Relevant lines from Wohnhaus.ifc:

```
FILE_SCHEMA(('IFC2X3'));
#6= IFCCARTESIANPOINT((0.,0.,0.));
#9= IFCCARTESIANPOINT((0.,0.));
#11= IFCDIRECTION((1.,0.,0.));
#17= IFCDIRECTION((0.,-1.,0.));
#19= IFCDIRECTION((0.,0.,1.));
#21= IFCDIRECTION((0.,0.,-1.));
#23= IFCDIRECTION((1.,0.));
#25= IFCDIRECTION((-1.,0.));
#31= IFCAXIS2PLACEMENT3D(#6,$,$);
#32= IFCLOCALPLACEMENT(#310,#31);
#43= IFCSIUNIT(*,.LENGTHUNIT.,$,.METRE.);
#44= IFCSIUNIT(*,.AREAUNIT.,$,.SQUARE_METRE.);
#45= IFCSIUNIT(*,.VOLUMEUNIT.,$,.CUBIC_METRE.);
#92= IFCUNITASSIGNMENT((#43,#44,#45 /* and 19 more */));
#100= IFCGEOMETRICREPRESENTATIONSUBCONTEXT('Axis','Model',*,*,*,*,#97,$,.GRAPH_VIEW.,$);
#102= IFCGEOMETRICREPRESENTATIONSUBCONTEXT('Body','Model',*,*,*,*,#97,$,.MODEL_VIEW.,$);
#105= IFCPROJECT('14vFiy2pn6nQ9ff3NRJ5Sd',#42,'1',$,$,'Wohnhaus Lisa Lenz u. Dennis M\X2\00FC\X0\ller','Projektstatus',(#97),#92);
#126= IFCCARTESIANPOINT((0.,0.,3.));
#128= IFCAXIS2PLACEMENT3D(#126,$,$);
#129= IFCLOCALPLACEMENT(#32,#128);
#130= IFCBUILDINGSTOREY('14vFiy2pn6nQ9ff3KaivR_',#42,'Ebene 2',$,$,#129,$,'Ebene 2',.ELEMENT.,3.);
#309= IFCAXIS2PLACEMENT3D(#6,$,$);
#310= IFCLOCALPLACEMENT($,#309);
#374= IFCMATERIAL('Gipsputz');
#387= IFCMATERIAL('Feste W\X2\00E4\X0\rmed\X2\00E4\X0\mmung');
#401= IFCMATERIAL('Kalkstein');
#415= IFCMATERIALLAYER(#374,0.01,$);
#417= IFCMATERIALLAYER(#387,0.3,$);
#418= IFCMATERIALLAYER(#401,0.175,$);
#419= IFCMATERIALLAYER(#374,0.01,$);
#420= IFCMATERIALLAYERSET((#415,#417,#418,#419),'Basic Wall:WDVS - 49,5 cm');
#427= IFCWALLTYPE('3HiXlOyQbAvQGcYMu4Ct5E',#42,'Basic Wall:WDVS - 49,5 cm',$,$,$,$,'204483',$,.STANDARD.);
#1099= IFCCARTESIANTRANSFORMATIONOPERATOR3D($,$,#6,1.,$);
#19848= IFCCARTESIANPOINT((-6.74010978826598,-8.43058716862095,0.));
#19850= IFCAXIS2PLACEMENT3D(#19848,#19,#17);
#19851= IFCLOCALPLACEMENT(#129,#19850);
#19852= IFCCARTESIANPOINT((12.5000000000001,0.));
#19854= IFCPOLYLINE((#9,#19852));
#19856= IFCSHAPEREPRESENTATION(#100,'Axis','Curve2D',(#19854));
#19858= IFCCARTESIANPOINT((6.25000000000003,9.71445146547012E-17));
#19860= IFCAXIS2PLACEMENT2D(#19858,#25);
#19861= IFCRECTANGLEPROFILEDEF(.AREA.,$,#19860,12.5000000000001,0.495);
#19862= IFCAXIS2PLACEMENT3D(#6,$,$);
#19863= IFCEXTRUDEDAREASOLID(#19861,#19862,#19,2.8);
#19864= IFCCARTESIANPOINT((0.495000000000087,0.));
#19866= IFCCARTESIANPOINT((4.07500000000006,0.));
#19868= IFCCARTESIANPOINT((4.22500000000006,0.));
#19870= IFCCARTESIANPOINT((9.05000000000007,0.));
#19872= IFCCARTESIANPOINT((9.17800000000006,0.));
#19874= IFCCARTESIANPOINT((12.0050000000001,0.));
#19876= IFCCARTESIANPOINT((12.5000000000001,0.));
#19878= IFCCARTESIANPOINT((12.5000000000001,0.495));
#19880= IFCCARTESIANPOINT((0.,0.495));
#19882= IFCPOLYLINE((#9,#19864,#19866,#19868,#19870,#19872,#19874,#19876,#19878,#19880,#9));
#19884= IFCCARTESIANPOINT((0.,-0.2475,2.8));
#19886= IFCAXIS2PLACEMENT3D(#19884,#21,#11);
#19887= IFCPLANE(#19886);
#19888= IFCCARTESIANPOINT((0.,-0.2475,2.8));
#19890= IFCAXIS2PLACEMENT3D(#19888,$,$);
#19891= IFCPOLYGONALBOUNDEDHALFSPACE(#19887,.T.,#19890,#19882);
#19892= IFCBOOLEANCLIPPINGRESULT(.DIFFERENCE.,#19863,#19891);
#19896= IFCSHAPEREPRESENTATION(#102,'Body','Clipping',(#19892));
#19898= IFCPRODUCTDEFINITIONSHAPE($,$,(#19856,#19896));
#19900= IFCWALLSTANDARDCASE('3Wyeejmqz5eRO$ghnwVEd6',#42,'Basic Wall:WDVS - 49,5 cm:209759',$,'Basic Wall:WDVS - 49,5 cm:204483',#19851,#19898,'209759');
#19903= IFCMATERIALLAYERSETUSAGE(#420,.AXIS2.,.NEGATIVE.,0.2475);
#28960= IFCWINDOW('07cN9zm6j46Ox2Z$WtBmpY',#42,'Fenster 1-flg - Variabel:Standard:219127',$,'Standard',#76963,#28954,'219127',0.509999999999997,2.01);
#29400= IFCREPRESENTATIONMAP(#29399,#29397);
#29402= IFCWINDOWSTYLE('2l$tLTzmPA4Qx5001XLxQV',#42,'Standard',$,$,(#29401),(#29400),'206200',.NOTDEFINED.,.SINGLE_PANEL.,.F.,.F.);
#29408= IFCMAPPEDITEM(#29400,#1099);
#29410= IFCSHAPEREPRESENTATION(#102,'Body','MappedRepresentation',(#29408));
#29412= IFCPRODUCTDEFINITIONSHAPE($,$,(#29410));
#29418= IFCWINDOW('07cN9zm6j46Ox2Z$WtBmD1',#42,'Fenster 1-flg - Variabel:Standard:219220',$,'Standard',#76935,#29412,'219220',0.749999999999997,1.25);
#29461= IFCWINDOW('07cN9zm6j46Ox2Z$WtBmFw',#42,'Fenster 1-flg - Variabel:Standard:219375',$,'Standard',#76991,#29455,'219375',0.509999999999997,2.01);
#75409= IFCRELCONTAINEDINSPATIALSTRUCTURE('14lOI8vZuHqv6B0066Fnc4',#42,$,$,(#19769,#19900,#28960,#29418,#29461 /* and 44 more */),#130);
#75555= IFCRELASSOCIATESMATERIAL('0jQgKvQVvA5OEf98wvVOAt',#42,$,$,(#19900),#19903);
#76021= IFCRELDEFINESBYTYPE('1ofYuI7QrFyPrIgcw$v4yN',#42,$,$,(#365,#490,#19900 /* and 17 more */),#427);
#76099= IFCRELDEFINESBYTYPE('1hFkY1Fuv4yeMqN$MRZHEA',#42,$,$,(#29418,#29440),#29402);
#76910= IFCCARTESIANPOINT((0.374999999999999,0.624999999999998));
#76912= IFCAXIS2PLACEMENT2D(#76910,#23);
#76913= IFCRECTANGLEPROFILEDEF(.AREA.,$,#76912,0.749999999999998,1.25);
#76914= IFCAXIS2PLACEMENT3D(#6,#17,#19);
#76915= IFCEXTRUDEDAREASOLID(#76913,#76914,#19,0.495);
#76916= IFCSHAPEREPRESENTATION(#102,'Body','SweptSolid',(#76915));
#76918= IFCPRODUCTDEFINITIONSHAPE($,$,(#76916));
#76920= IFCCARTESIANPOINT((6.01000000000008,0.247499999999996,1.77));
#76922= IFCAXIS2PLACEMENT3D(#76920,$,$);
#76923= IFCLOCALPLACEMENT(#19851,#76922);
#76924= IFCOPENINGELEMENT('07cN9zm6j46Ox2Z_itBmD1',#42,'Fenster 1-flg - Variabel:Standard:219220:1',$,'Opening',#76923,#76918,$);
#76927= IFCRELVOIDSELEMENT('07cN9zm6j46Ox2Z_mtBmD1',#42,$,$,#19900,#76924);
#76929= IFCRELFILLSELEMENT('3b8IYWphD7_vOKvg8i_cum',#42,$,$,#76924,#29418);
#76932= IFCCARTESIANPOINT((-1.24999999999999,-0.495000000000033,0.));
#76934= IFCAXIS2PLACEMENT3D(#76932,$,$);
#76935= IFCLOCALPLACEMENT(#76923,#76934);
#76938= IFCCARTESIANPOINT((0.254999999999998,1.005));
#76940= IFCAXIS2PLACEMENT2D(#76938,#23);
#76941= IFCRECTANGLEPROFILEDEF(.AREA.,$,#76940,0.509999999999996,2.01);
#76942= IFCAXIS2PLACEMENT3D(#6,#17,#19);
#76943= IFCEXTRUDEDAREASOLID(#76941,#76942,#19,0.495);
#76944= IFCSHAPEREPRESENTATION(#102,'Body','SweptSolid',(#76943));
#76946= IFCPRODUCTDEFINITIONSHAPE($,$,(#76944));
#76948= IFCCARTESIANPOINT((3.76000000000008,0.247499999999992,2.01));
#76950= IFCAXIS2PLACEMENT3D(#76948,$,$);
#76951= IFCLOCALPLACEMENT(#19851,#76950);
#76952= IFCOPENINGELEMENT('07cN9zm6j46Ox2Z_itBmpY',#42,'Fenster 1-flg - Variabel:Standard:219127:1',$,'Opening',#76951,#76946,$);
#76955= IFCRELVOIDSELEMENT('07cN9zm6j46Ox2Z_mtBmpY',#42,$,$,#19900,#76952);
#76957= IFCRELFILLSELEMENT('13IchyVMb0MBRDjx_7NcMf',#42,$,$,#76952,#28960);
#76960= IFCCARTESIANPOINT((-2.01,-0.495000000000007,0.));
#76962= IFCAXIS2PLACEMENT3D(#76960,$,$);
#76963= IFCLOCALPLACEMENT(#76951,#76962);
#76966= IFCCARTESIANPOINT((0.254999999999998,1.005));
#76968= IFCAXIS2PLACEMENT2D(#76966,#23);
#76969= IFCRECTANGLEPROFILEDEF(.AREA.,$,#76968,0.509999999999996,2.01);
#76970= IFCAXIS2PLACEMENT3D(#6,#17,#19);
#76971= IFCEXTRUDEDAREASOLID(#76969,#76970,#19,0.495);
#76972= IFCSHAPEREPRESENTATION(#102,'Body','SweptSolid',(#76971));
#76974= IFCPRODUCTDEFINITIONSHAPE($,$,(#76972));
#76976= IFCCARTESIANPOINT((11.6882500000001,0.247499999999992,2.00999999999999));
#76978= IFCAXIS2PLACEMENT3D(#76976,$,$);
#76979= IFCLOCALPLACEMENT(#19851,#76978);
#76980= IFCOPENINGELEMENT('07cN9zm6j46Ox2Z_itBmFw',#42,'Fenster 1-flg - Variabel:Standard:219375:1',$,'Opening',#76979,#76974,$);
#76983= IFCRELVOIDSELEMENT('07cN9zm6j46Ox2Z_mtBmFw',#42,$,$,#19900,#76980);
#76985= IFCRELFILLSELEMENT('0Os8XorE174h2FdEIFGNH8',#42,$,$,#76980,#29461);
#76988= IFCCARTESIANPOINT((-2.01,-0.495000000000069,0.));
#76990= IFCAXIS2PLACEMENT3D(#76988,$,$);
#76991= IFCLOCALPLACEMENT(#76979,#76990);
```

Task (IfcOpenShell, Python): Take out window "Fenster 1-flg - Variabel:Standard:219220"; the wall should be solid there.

```python
import ifcopenshell
import ifcopenshell.api.feature
import ifcopenshell.api.root
import ifcopenshell.geom
import ifcopenshell.util.shape

model = ifcopenshell.open("Wohnhaus.ifc")
settings = ifcopenshell.geom.settings()


def volume(element):
    """Net volume in cubic metres, openings subtracted."""
    shape = ifcopenshell.geom.create_shape(settings, element)
    return ifcopenshell.util.shape.get_volume(shape.geometry)


window = model.by_guid("07cN9zm6j46Ox2Z$WtBmD1")
opening = window.FillsVoids[0].RelatingOpeningElement
wall = opening.VoidsElements[0].RelatingBuildingElement
before = volume(wall)

ifcopenshell.api.root.remove_product(model, product=window)
ifcopenshell.api.feature.remove_feature(model, feature=opening)

after = volume(wall)

print(f"wall volume {before:.3f} -> {after:.3f} m3")

model.write("Wohnhaus-out.ifc")
```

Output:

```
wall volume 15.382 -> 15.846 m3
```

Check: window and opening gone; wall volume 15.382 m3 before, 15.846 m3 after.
